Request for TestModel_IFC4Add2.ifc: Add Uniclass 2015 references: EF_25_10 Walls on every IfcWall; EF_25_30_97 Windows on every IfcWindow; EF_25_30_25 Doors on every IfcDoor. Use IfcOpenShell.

First a look at what the model holds.

```python
import ifcopenshell

model = ifcopenshell.open("TestModel_IFC4Add2.ifc")
print(model.schema)
print("classifications:", [c.Name for c in model.by_type("IfcClassification")])
for ifc_class in ("IfcDoor", "IfcRoof", "IfcStair", "IfcWall", "IfcWindow"):
    print(ifc_class, len(model.by_type(ifc_class)))
```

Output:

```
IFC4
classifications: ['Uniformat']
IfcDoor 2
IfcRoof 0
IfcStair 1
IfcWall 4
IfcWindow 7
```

```python
import ifcopenshell
import ifcopenshell.api.classification

model = ifcopenshell.open("TestModel_IFC4Add2.ifc")

system = ifcopenshell.api.classification.add_classification(model, classification="Uniclass 2015")

codes = {
    "IfcWall": ("EF_25_10", "Walls"),
    "IfcWindow": ("EF_25_30_97", "Windows"),
    "IfcDoor": ("EF_25_30_25", "Doors"),
}
for ifc_class, (code, name) in codes.items():
    products = model.by_type(ifc_class)
    ifcopenshell.api.classification.add_reference(
        model, products=products, classification=system, identification=code, name=name
    )
    print(code, len(products))

model.write("TestModel_IFC4Add2_rev.ifc")
```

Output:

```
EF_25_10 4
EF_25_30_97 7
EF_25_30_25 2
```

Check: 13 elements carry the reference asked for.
